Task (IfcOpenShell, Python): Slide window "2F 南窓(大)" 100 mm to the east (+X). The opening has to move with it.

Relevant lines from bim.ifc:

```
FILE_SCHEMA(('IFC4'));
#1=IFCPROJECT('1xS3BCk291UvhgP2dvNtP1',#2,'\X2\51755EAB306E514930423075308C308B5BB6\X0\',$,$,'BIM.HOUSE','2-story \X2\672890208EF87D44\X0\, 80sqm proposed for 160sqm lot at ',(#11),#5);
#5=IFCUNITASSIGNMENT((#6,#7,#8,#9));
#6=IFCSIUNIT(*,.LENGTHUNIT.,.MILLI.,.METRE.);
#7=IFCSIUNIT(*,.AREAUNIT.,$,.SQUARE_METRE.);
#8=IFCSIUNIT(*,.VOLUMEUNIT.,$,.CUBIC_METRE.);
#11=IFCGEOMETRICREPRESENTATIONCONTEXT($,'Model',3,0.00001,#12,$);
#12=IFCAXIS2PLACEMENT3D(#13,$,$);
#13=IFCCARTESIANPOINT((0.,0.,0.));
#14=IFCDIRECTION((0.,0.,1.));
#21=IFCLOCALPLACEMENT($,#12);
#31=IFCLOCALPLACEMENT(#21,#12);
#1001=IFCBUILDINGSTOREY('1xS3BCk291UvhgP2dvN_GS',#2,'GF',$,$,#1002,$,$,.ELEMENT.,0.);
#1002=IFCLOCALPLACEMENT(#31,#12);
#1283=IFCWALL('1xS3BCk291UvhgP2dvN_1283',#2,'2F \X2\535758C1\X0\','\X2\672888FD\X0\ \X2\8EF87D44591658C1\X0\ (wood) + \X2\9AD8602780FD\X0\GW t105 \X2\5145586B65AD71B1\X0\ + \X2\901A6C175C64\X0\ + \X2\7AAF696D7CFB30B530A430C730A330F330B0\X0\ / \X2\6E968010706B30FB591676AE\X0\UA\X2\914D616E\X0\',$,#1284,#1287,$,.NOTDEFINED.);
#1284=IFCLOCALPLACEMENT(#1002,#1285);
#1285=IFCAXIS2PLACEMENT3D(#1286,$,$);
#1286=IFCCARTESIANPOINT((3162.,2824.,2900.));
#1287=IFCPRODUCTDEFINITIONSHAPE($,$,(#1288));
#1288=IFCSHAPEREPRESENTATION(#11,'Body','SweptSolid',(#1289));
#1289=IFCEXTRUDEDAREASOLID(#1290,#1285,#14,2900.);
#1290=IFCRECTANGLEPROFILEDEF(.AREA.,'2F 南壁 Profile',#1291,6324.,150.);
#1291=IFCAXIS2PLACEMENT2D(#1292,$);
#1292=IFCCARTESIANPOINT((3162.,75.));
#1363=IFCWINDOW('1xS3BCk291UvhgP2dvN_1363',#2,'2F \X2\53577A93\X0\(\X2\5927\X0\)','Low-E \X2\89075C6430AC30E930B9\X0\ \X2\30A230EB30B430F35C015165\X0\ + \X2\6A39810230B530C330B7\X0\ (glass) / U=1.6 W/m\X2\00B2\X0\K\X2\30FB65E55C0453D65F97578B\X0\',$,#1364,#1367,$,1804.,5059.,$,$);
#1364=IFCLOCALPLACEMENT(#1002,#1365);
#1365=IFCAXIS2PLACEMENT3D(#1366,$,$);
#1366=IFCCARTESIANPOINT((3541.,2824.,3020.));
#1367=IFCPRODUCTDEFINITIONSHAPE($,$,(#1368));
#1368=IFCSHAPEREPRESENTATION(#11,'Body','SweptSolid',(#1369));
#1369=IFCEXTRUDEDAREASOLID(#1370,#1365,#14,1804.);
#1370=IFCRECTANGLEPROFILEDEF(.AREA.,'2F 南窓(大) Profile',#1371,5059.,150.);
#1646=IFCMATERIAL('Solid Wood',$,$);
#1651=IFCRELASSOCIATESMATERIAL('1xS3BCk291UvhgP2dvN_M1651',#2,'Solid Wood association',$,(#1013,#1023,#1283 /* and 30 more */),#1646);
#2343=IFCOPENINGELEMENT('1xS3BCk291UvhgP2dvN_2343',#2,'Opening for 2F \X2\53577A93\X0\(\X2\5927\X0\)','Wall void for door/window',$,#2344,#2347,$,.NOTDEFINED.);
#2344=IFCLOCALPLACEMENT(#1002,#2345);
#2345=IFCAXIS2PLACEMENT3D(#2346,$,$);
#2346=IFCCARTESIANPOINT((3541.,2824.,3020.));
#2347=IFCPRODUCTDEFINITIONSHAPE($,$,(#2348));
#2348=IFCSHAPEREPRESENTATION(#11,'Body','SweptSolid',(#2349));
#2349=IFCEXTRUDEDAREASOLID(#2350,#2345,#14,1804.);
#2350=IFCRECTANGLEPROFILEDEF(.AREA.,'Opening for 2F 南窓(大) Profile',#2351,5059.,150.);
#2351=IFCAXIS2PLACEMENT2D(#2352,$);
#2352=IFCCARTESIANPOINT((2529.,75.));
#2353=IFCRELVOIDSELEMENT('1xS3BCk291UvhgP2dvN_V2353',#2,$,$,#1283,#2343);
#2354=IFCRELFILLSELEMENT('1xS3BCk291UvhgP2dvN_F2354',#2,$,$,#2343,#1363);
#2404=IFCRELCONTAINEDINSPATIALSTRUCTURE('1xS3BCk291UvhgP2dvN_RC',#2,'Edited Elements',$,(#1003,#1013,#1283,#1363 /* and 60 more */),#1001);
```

```python
import ifcopenshell
import ifcopenshell.api.geometry
import ifcopenshell.util.placement
import ifcopenshell.util.unit

model = ifcopenshell.open("bim.ifc")
unit_scale = ifcopenshell.util.unit.calculate_unit_scale(model)

window = model.by_guid("1xS3BCk291UvhgP2dvN_1363")
opening = window.FillsVoids[0].RelatingOpeningElement
wall = opening.VoidsElements[0].RelatingBuildingElement

wall_matrix = ifcopenshell.util.placement.get_local_placement(wall.ObjectPlacement)
shift = wall_matrix[:3, 0] * 0.1 / unit_scale
before = ifcopenshell.util.placement.get_local_placement(window.ObjectPlacement)[:3, 3].copy()

# The window is not placed relative to its opening, so move both.
for product in (opening, window):
    matrix = ifcopenshell.util.placement.get_local_placement(product.ObjectPlacement)
    matrix[:3, 3] += shift
    ifcopenshell.api.geometry.edit_object_placement(model, product=product, matrix=matrix, is_si=False)

after = ifcopenshell.util.placement.get_local_placement(window.ObjectPlacement)[:3, 3]
print("window moved by", (after - before).round(3) + 0.0)

model.write("bim-out.ifc")
```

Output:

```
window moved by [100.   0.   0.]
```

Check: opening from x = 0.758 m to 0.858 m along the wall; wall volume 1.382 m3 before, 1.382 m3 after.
